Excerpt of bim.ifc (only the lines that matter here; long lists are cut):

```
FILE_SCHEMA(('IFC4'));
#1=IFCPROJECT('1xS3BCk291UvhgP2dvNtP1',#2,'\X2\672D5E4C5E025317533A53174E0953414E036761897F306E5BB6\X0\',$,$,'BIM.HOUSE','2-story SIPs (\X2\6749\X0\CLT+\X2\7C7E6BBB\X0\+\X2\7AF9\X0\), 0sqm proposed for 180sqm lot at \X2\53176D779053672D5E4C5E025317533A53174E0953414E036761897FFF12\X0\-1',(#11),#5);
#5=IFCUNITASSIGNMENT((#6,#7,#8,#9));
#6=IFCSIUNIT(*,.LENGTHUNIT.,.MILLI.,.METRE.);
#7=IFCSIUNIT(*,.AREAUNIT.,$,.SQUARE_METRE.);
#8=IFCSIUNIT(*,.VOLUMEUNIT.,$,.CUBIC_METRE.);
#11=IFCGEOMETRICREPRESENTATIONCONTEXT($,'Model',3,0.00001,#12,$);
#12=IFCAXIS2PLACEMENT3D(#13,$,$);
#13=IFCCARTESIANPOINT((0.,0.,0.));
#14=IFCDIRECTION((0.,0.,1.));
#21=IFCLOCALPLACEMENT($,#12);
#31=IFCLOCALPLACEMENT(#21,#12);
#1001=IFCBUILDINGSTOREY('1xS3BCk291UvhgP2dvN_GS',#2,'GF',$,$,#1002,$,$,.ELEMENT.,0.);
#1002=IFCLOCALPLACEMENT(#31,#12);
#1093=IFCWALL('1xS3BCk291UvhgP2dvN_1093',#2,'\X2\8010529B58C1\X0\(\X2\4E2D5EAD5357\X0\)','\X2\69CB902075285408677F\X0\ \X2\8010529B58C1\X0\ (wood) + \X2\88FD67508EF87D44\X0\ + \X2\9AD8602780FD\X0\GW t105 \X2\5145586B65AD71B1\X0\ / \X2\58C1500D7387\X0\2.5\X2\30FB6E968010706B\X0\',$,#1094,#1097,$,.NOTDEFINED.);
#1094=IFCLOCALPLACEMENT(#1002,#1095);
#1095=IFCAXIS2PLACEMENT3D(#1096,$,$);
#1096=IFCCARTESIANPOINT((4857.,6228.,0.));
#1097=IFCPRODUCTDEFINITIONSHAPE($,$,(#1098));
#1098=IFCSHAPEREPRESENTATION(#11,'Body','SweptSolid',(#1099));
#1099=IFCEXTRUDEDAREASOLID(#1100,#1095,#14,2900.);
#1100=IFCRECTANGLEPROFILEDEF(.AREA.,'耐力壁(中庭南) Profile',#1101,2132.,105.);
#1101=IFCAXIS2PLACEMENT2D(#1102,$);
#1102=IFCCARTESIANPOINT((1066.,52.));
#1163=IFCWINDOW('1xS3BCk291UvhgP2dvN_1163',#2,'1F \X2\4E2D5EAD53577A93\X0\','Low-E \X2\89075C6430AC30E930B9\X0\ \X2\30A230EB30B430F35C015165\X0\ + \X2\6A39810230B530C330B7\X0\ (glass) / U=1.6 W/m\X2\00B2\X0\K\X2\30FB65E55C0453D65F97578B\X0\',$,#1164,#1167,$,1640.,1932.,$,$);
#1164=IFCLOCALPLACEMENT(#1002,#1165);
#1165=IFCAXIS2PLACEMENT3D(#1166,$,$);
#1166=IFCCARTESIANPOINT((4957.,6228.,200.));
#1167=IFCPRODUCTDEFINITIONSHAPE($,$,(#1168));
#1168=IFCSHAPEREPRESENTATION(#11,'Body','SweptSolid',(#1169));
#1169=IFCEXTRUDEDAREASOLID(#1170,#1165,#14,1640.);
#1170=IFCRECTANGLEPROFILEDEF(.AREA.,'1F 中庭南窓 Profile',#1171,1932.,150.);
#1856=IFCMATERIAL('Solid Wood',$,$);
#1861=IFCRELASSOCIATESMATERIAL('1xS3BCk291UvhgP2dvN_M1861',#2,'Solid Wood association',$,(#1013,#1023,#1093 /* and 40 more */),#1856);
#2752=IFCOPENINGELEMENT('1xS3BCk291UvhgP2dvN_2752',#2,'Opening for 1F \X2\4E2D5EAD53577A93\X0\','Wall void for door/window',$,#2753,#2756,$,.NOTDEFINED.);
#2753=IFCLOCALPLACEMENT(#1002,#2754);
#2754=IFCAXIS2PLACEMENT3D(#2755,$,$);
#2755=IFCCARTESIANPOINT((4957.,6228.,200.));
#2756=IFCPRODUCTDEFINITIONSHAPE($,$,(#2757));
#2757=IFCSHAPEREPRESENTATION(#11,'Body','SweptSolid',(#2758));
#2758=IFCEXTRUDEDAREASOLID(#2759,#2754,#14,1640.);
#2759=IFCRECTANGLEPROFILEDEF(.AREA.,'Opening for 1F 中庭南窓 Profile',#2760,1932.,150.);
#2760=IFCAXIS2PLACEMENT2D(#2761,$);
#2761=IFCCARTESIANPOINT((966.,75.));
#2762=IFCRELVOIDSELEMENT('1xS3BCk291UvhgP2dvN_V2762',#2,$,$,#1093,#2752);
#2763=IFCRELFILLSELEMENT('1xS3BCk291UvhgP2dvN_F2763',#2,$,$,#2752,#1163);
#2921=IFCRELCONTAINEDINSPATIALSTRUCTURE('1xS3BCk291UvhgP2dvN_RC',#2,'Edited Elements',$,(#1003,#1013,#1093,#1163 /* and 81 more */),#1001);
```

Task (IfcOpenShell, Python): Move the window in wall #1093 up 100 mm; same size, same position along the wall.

```python
import numpy as np
import ifcopenshell
import ifcopenshell.api.geometry
import ifcopenshell.util.placement
import ifcopenshell.util.unit

model = ifcopenshell.open("bim.ifc")
unit_scale = ifcopenshell.util.unit.calculate_unit_scale(model)

window = model.by_guid("1xS3BCk291UvhgP2dvN_1163")
opening = window.FillsVoids[0].RelatingOpeningElement
dz = 0.1 / unit_scale

shift = np.array([0.0, 0.0, dz])
# The window is not placed relative to its opening, so move both.
for product in (opening, window):
    matrix = ifcopenshell.util.placement.get_local_placement(product.ObjectPlacement)
    matrix[:3, 3] += shift
    ifcopenshell.api.geometry.edit_object_placement(model, product=product, matrix=matrix, is_si=False)

print(f"moved by {dz * unit_scale:+.3f} m")

model.write("bim-out.ifc")
```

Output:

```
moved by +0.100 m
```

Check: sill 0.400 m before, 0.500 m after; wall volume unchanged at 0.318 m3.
